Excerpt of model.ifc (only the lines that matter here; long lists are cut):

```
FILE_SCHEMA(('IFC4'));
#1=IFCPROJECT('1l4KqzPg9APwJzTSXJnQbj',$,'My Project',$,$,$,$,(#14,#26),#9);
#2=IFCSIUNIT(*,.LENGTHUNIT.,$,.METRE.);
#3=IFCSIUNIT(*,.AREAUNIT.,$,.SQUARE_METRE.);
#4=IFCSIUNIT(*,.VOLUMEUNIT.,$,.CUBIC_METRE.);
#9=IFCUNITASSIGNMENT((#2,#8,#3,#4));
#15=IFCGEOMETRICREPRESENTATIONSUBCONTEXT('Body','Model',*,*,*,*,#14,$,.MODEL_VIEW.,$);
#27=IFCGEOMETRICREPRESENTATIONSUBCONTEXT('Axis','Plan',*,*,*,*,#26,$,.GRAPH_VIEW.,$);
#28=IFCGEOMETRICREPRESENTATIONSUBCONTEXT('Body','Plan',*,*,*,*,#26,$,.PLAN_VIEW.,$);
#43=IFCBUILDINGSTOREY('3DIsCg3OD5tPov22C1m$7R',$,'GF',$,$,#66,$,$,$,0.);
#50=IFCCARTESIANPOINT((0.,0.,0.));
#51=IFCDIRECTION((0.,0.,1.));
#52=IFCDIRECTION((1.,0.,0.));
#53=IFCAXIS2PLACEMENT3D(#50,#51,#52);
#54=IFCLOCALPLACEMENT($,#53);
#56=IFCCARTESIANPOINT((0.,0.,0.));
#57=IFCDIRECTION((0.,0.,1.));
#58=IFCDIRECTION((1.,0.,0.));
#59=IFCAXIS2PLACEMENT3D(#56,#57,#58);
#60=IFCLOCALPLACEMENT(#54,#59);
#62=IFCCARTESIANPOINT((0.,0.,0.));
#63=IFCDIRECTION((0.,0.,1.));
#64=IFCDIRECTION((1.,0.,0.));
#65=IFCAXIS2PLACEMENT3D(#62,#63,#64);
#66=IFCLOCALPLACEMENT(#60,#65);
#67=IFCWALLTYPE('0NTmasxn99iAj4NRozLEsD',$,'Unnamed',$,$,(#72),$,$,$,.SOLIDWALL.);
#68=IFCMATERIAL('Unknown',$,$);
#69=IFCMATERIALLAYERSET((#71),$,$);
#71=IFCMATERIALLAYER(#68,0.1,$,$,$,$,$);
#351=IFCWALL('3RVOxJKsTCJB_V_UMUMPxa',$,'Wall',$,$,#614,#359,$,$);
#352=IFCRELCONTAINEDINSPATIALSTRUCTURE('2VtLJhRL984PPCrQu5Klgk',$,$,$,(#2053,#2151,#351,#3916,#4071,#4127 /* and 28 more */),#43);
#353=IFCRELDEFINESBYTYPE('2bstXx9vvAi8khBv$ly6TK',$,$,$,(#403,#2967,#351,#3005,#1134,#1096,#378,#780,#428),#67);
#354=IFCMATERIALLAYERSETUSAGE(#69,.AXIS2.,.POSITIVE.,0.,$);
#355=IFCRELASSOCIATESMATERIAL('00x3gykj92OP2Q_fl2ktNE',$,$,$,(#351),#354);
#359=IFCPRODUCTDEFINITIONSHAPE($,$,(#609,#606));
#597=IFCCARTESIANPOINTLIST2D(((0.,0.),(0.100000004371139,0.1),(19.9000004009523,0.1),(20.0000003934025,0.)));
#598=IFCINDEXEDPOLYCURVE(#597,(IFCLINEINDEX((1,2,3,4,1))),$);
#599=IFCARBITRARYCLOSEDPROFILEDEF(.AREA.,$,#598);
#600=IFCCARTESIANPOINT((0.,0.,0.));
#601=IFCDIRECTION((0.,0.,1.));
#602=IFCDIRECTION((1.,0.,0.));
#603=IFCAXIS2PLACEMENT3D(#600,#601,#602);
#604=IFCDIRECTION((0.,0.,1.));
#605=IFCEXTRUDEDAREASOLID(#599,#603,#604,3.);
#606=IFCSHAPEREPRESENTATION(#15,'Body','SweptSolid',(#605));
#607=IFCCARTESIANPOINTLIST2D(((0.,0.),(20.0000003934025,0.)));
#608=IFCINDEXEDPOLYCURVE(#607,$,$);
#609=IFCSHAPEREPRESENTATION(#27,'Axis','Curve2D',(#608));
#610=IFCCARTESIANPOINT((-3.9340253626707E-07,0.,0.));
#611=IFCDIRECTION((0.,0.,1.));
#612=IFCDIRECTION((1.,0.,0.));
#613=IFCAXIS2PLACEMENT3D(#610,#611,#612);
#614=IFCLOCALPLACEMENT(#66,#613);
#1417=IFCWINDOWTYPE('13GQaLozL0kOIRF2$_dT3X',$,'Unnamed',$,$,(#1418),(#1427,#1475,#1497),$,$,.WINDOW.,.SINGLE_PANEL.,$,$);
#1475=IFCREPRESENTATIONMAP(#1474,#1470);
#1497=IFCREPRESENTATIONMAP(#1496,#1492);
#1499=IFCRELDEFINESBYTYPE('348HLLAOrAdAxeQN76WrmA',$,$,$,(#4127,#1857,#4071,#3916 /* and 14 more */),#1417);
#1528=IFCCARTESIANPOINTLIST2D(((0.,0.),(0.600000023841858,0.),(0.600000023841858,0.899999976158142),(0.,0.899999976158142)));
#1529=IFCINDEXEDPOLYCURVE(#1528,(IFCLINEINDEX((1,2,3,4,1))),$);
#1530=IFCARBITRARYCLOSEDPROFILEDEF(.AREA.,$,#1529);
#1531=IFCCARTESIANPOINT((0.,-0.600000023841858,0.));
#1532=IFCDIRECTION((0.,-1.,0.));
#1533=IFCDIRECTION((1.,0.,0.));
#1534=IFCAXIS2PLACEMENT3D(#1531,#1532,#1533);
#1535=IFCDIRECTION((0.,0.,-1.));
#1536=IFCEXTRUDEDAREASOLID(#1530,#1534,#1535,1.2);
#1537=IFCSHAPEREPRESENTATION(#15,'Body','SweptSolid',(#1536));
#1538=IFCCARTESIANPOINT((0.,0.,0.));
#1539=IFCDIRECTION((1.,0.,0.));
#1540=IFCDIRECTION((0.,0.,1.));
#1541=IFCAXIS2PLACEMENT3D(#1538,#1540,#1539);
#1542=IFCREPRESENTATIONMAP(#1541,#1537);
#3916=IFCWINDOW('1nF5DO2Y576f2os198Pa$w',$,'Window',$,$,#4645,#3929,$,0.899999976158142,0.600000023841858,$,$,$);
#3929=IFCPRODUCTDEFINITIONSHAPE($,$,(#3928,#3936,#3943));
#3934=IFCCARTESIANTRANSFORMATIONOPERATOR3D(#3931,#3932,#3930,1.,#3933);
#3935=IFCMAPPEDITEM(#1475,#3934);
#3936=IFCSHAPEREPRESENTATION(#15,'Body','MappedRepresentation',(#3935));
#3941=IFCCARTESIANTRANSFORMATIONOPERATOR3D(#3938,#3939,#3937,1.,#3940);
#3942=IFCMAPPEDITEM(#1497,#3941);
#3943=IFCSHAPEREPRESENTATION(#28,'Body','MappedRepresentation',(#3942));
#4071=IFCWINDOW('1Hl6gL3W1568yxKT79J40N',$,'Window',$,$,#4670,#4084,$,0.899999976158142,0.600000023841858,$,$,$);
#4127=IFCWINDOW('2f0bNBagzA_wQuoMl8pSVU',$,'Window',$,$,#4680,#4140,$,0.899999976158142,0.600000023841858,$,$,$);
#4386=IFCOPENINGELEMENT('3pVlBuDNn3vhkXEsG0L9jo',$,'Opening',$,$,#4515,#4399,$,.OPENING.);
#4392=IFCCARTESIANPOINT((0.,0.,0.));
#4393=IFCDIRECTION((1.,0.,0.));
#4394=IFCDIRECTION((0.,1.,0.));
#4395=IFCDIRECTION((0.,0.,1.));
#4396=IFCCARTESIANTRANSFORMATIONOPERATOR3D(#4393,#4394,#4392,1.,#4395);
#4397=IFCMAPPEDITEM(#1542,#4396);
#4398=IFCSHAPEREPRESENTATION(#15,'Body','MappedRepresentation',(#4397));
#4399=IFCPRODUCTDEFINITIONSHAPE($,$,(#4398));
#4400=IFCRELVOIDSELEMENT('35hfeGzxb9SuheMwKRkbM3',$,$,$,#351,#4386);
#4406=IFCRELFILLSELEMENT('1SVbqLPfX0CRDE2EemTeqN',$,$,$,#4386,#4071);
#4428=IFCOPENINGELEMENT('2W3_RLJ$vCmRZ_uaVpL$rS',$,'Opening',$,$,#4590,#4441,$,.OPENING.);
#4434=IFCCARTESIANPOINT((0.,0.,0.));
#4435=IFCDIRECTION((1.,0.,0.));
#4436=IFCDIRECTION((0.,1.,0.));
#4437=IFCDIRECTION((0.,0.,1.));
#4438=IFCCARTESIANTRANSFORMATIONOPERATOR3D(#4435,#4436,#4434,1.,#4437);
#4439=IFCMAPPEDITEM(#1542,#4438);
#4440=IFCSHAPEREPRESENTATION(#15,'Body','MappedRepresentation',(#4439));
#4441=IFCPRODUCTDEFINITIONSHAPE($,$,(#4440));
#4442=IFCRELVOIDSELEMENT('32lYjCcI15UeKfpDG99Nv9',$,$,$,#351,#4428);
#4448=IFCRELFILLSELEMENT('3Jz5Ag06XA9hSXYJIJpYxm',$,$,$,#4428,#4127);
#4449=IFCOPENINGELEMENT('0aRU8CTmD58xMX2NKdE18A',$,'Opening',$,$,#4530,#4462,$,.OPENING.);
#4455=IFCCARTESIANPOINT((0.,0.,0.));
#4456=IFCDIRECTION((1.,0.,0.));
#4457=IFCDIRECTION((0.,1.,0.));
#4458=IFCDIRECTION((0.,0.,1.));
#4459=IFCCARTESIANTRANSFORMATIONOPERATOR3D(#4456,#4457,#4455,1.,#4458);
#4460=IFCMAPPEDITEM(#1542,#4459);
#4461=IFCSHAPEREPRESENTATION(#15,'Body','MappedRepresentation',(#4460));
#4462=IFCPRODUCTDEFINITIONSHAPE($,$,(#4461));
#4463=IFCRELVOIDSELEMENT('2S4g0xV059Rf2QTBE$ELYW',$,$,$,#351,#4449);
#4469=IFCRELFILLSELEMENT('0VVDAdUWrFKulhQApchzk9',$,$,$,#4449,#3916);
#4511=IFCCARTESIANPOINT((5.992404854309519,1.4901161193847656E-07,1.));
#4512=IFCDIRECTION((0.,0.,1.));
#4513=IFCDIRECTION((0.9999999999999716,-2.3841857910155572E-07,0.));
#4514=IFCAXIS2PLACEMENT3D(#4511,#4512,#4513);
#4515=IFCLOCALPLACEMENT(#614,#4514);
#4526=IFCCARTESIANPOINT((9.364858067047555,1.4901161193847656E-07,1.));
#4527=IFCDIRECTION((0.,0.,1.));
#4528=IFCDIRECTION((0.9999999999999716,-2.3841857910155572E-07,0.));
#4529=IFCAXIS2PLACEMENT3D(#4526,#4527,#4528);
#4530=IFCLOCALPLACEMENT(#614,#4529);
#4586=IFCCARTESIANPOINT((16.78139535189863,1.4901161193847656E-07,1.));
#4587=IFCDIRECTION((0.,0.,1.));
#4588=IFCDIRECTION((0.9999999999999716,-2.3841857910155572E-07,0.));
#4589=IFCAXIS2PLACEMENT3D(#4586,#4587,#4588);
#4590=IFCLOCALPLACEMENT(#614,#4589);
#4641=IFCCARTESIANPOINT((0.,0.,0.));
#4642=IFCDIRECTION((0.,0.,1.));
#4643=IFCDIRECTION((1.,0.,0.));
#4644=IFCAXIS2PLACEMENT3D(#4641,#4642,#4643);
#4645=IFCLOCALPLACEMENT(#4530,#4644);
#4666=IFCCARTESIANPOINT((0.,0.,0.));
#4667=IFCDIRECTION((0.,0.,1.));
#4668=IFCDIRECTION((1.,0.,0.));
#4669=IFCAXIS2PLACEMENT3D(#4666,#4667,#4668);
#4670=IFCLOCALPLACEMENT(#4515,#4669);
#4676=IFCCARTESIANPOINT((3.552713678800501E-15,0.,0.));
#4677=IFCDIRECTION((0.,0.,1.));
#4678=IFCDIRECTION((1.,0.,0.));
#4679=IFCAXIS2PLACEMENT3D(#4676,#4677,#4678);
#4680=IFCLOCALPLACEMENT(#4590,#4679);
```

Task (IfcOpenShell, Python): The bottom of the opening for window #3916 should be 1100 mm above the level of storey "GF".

```python
import numpy as np
import ifcopenshell
import ifcopenshell.api.geometry
import ifcopenshell.geom
import ifcopenshell.util.element
import ifcopenshell.util.placement
import ifcopenshell.util.shape
import ifcopenshell.util.unit

model = ifcopenshell.open("model.ifc")
unit_scale = ifcopenshell.util.unit.calculate_unit_scale(model)

window = model.by_guid("1nF5DO2Y576f2os198Pa$w")
opening = window.FillsVoids[0].RelatingOpeningElement
storey = ifcopenshell.util.element.get_container(window, ifc_class="IfcBuildingStorey")
level = ifcopenshell.util.placement.get_local_placement(storey.ObjectPlacement)[2, 3]

# The opening's origin need not be at the sill, so measure its lowest point.
shape = ifcopenshell.geom.create_shape(ifcopenshell.geom.settings(), opening)
bottom = ifcopenshell.util.shape.get_shape_bottom_elevation(shape, shape.geometry) / unit_scale
dz = level + 1.1 / unit_scale - bottom

shift = np.array([0.0, 0.0, dz])
# The window is placed relative to its opening, so it follows when the opening moves.
matrix = ifcopenshell.util.placement.get_local_placement(opening.ObjectPlacement)
matrix[:3, 3] += shift
ifcopenshell.api.geometry.edit_object_placement(
    model, product=opening, matrix=matrix, is_si=False, should_transform_children=True
)

print(f"moved by {dz * unit_scale:+.3f} m")

model.write("model_v2.ifc")
```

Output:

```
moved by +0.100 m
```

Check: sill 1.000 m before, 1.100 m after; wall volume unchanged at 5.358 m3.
